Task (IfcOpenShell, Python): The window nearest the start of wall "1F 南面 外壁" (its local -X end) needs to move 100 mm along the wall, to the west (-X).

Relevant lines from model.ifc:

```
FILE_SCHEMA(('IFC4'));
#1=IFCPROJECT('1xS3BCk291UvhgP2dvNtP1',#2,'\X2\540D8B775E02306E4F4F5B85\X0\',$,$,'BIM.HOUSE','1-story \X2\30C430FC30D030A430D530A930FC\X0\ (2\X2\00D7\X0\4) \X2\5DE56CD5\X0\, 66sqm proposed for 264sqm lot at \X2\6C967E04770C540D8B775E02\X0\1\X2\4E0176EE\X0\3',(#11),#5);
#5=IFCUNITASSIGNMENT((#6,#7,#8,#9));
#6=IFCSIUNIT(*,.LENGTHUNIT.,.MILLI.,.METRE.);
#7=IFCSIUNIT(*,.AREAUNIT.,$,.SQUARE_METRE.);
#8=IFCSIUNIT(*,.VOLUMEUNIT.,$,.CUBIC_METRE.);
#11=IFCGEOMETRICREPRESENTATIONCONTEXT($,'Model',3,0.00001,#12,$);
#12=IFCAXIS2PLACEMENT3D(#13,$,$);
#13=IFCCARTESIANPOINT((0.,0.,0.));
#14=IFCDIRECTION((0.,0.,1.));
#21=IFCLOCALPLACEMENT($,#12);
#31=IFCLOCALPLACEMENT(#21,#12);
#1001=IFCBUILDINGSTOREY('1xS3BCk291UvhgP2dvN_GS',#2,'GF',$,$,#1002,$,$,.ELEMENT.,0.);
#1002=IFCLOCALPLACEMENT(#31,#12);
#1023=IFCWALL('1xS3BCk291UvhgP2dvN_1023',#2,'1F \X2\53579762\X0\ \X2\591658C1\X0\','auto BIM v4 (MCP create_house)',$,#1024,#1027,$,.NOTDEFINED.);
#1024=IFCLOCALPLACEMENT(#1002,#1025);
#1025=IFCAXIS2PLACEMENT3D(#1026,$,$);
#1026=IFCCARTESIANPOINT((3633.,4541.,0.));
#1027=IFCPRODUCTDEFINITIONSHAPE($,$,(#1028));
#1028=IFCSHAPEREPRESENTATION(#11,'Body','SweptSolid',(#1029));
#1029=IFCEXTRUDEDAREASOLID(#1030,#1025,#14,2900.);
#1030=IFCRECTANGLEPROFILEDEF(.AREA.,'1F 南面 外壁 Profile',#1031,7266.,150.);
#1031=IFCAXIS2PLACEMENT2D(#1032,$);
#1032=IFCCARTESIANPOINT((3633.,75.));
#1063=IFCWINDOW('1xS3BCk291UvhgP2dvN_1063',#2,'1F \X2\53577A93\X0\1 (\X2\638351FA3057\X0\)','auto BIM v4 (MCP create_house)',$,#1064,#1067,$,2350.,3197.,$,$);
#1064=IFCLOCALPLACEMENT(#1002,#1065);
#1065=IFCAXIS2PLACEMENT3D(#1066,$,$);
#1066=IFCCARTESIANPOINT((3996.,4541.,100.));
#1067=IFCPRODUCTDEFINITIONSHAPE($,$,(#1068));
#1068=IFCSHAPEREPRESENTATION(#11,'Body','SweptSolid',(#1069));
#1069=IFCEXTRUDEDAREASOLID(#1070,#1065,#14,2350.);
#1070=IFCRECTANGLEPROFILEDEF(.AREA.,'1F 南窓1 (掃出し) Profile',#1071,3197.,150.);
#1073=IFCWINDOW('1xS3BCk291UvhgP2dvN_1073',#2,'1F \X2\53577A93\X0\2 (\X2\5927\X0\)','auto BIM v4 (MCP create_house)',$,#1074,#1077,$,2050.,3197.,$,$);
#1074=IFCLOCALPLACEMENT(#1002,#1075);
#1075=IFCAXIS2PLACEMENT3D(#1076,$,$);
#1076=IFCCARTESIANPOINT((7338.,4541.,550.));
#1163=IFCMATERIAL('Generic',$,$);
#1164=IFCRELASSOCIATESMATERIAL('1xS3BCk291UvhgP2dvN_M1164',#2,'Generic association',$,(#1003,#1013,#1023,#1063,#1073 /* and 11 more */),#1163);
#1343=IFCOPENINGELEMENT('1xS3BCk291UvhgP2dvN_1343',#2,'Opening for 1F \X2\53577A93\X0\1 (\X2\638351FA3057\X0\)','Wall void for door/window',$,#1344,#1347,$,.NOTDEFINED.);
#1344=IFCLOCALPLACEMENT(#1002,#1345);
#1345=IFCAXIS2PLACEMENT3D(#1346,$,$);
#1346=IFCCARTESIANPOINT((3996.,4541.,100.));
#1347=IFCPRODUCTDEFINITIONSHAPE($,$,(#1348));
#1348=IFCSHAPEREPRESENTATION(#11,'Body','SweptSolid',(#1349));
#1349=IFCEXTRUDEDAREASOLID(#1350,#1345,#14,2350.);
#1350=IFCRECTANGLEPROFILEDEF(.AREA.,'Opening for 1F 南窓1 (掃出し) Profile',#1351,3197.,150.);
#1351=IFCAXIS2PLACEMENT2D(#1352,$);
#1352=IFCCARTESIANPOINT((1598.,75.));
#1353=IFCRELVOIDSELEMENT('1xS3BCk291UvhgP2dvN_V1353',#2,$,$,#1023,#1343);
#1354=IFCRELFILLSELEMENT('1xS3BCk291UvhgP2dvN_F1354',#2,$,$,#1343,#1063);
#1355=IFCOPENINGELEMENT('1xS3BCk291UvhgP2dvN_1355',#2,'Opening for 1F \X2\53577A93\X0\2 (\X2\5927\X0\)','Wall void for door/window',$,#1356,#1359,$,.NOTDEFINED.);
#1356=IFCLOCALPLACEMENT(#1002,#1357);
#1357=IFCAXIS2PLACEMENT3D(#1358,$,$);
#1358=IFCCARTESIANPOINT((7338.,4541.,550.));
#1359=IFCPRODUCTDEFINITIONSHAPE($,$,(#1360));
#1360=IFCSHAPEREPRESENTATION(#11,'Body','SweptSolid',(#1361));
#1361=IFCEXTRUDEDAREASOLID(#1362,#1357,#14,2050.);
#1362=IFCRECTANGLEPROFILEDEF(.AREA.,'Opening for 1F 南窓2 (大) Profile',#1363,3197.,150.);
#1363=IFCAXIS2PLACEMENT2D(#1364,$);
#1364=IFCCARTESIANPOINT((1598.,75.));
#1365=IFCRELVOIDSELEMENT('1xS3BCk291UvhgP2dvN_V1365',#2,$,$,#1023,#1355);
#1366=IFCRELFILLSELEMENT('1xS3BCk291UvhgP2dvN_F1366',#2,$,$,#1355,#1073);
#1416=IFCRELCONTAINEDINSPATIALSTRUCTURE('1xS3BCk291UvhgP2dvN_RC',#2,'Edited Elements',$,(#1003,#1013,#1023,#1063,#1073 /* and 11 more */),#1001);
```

```python
import ifcopenshell
import ifcopenshell.api.geometry
import ifcopenshell.util.placement
import ifcopenshell.util.unit

model = ifcopenshell.open("model.ifc")
unit_scale = ifcopenshell.util.unit.calculate_unit_scale(model)

window = model.by_guid("1xS3BCk291UvhgP2dvN_1063")
opening = window.FillsVoids[0].RelatingOpeningElement
wall = opening.VoidsElements[0].RelatingBuildingElement

wall_matrix = ifcopenshell.util.placement.get_local_placement(wall.ObjectPlacement)
shift = wall_matrix[:3, 0] * -0.1 / unit_scale
before = ifcopenshell.util.placement.get_local_placement(window.ObjectPlacement)[:3, 3].copy()

# The window is not placed relative to its opening, so move both.
for product in (opening, window):
    matrix = ifcopenshell.util.placement.get_local_placement(product.ObjectPlacement)
    matrix[:3, 3] += shift
    ifcopenshell.api.geometry.edit_object_placement(model, product=product, matrix=matrix, is_si=False)

after = ifcopenshell.util.placement.get_local_placement(window.ObjectPlacement)[:3, 3]
print("window moved by", (after - before).round(3) + 0.0)

model.write("model_edited.ifc")
```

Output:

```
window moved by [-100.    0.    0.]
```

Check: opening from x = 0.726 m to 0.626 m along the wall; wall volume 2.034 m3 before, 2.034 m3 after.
